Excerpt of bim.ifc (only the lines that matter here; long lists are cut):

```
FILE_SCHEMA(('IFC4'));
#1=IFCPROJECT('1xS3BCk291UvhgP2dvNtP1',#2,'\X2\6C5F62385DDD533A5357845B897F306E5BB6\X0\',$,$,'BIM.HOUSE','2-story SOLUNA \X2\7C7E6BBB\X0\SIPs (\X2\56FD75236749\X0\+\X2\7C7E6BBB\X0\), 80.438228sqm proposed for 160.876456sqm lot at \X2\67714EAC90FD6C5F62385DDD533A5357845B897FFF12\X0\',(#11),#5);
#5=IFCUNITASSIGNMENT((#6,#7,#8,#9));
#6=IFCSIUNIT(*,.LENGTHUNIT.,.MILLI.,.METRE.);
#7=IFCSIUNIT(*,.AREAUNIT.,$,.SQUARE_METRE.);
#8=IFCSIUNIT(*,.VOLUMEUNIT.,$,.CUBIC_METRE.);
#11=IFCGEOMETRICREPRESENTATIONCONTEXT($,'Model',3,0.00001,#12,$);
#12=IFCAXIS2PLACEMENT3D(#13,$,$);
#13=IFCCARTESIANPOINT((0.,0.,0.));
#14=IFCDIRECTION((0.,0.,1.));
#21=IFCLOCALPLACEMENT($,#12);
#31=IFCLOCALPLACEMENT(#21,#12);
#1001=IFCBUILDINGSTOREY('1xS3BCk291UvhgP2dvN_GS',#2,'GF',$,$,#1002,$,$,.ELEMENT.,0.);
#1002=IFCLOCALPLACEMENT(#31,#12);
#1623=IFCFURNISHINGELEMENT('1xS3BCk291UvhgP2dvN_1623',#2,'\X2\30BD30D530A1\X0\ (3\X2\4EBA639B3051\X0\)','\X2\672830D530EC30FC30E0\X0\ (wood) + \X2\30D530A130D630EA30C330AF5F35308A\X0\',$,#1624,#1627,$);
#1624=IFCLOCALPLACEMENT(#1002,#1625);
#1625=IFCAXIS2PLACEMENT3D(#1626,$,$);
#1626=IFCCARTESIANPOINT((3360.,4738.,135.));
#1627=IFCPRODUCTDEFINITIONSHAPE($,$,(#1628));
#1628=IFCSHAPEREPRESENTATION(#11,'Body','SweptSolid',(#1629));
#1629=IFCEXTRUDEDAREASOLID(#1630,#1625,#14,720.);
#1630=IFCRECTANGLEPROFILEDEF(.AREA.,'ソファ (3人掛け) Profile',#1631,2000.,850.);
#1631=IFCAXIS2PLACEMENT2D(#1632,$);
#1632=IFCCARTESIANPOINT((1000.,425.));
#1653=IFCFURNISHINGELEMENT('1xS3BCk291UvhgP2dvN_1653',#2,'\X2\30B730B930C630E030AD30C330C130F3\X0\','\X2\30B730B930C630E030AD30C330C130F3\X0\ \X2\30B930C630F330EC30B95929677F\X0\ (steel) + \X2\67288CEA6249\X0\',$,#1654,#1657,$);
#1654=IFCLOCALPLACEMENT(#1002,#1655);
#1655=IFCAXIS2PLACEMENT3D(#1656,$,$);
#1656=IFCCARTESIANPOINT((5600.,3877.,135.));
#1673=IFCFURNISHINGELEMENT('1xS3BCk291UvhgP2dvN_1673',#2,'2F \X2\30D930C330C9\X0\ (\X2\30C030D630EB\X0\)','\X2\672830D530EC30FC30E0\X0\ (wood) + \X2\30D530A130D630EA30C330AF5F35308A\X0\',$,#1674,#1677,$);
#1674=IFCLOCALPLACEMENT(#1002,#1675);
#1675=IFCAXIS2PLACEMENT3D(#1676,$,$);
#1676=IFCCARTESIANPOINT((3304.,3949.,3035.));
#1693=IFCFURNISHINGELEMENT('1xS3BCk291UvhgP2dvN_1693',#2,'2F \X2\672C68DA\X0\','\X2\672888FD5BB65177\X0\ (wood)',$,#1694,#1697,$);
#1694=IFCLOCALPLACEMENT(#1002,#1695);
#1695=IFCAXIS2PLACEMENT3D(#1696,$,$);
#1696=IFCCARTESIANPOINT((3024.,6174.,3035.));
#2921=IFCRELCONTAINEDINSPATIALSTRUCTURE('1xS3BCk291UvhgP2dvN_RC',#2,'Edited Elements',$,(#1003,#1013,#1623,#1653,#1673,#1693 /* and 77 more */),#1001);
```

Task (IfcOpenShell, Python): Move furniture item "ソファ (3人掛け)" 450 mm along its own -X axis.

```python
import ifcopenshell
import ifcopenshell.api.geometry
import ifcopenshell.util.placement

model = ifcopenshell.open("bim.ifc")

item = model.by_guid("1xS3BCk291UvhgP2dvN_1623")
matrix = ifcopenshell.util.placement.get_local_placement(item.ObjectPlacement)
matrix[:3, 3] -= matrix[:3, 0] * 450.0
ifcopenshell.api.geometry.edit_object_placement(model, product=item, matrix=matrix, is_si=False)

print(ifcopenshell.util.placement.get_local_placement(item.ObjectPlacement).round(3) + 0.0)

model.write("bim_updated.ifc")
```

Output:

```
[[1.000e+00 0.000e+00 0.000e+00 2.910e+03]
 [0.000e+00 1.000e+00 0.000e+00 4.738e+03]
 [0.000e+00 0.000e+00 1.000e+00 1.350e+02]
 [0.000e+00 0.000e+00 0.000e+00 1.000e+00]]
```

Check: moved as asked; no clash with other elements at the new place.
